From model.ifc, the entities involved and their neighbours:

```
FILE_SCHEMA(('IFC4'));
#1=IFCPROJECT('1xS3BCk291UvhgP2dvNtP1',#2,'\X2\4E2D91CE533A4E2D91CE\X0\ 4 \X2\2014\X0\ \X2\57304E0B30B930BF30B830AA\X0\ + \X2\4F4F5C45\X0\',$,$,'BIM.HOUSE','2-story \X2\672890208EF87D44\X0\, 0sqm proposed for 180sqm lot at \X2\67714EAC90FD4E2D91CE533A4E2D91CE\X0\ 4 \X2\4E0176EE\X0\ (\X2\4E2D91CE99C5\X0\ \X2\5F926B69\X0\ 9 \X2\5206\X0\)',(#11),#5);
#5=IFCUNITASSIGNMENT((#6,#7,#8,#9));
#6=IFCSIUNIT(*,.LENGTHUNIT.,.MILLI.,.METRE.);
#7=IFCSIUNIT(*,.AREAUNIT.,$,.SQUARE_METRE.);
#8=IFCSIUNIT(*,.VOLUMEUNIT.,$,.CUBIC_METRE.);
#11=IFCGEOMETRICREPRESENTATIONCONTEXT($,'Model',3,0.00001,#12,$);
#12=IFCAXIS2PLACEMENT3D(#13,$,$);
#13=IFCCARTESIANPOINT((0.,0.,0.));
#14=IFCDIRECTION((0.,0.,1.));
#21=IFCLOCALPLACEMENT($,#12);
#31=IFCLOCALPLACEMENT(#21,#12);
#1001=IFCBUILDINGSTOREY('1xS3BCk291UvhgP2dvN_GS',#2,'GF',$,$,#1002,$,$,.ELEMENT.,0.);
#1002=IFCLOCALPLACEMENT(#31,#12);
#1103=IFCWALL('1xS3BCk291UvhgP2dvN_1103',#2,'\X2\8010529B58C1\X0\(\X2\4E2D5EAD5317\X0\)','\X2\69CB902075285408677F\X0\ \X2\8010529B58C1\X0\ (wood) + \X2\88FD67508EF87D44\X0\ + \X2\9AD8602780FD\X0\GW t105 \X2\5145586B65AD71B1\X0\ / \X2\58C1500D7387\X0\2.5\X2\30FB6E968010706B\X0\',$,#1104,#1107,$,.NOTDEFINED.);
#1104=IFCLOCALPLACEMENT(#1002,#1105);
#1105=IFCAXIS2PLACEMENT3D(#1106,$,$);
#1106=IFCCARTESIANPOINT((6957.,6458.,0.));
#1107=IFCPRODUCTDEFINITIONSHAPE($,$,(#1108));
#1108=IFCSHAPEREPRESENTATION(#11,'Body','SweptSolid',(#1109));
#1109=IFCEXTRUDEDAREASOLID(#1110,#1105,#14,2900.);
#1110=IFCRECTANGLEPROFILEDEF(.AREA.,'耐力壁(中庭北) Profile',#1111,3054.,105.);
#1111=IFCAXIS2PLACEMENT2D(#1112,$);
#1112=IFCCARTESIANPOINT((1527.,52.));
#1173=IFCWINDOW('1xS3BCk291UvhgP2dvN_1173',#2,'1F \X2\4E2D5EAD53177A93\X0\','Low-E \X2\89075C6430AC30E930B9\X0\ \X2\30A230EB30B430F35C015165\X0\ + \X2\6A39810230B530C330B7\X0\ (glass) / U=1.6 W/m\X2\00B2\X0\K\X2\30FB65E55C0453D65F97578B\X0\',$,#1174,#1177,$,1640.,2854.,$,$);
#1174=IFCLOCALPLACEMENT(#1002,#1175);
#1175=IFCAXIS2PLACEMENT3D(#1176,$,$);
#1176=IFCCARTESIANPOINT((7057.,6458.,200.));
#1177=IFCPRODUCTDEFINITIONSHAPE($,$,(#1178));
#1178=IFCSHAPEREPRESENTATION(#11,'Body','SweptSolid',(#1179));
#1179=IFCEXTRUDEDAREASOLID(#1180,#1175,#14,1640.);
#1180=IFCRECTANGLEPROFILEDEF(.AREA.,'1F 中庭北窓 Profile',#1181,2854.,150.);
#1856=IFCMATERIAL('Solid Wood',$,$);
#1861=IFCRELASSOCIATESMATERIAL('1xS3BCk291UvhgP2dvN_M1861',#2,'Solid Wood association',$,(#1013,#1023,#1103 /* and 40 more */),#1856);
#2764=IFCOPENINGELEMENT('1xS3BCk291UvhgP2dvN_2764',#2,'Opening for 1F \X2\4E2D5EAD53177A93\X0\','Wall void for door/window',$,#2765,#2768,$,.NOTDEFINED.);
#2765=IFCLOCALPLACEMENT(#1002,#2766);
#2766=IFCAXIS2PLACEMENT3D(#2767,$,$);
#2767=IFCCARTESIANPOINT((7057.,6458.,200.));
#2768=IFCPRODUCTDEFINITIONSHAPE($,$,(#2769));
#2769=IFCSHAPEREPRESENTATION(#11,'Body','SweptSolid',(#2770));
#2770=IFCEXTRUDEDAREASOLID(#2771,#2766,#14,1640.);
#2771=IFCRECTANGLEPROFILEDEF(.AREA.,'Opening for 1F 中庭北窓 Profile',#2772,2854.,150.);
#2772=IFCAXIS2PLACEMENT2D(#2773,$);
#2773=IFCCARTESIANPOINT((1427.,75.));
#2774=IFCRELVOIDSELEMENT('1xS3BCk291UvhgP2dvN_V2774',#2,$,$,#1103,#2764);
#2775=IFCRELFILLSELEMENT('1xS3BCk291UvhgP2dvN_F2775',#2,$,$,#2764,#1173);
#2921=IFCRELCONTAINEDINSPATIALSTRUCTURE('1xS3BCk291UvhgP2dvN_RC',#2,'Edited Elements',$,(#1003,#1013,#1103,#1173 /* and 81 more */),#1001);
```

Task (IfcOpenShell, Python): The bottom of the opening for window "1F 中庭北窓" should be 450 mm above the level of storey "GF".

```python
import numpy as np
import ifcopenshell
import ifcopenshell.api.geometry
import ifcopenshell.geom
import ifcopenshell.util.element
import ifcopenshell.util.placement
import ifcopenshell.util.shape
import ifcopenshell.util.unit

model = ifcopenshell.open("model.ifc")
unit_scale = ifcopenshell.util.unit.calculate_unit_scale(model)

window = model.by_guid("1xS3BCk291UvhgP2dvN_1173")
opening = window.FillsVoids[0].RelatingOpeningElement
storey = ifcopenshell.util.element.get_container(window, ifc_class="IfcBuildingStorey")
level = ifcopenshell.util.placement.get_local_placement(storey.ObjectPlacement)[2, 3]

# The opening's origin need not be at the sill, so measure its lowest point.
shape = ifcopenshell.geom.create_shape(ifcopenshell.geom.settings(), opening)
bottom = ifcopenshell.util.shape.get_shape_bottom_elevation(shape, shape.geometry) / unit_scale
dz = level + 450.0 - bottom

shift = np.array([0.0, 0.0, dz])
# The window is not placed relative to its opening, so move both.
for product in (opening, window):
    matrix = ifcopenshell.util.placement.get_local_placement(product.ObjectPlacement)
    matrix[:3, 3] += shift
    ifcopenshell.api.geometry.edit_object_placement(model, product=product, matrix=matrix, is_si=False)

print(f"moved by {dz * unit_scale:+.3f} m")

model.write("model_v2.ifc")
```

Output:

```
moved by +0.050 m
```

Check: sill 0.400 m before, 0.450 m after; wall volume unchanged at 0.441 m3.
